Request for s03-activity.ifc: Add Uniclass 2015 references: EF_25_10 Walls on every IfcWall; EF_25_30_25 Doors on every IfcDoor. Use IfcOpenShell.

First a look at what the model holds.

```python
import ifcopenshell

model = ifcopenshell.open("s03-activity.ifc")
print(model.schema)
print("classifications:", [c.Name for c in model.by_type("IfcClassification")])
for ifc_class in ("IfcDoor", "IfcRoof", "IfcStair", "IfcWall", "IfcWindow"):
    print(ifc_class, len(model.by_type(ifc_class)))
```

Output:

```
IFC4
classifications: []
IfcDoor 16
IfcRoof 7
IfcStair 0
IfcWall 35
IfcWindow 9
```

```python
import ifcopenshell
import ifcopenshell.api.classification

model = ifcopenshell.open("s03-activity.ifc")

system = ifcopenshell.api.classification.add_classification(model, classification="Uniclass 2015")

codes = {
    "IfcWall": ("EF_25_10", "Walls"),
    "IfcDoor": ("EF_25_30_25", "Doors"),
}
for ifc_class, (code, name) in codes.items():
    products = model.by_type(ifc_class)
    ifcopenshell.api.classification.add_reference(
        model, products=products, classification=system, identification=code, name=name
    )
    print(code, len(products))

model.write("s03-activity-out.ifc")
```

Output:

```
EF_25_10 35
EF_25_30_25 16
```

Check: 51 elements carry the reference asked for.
